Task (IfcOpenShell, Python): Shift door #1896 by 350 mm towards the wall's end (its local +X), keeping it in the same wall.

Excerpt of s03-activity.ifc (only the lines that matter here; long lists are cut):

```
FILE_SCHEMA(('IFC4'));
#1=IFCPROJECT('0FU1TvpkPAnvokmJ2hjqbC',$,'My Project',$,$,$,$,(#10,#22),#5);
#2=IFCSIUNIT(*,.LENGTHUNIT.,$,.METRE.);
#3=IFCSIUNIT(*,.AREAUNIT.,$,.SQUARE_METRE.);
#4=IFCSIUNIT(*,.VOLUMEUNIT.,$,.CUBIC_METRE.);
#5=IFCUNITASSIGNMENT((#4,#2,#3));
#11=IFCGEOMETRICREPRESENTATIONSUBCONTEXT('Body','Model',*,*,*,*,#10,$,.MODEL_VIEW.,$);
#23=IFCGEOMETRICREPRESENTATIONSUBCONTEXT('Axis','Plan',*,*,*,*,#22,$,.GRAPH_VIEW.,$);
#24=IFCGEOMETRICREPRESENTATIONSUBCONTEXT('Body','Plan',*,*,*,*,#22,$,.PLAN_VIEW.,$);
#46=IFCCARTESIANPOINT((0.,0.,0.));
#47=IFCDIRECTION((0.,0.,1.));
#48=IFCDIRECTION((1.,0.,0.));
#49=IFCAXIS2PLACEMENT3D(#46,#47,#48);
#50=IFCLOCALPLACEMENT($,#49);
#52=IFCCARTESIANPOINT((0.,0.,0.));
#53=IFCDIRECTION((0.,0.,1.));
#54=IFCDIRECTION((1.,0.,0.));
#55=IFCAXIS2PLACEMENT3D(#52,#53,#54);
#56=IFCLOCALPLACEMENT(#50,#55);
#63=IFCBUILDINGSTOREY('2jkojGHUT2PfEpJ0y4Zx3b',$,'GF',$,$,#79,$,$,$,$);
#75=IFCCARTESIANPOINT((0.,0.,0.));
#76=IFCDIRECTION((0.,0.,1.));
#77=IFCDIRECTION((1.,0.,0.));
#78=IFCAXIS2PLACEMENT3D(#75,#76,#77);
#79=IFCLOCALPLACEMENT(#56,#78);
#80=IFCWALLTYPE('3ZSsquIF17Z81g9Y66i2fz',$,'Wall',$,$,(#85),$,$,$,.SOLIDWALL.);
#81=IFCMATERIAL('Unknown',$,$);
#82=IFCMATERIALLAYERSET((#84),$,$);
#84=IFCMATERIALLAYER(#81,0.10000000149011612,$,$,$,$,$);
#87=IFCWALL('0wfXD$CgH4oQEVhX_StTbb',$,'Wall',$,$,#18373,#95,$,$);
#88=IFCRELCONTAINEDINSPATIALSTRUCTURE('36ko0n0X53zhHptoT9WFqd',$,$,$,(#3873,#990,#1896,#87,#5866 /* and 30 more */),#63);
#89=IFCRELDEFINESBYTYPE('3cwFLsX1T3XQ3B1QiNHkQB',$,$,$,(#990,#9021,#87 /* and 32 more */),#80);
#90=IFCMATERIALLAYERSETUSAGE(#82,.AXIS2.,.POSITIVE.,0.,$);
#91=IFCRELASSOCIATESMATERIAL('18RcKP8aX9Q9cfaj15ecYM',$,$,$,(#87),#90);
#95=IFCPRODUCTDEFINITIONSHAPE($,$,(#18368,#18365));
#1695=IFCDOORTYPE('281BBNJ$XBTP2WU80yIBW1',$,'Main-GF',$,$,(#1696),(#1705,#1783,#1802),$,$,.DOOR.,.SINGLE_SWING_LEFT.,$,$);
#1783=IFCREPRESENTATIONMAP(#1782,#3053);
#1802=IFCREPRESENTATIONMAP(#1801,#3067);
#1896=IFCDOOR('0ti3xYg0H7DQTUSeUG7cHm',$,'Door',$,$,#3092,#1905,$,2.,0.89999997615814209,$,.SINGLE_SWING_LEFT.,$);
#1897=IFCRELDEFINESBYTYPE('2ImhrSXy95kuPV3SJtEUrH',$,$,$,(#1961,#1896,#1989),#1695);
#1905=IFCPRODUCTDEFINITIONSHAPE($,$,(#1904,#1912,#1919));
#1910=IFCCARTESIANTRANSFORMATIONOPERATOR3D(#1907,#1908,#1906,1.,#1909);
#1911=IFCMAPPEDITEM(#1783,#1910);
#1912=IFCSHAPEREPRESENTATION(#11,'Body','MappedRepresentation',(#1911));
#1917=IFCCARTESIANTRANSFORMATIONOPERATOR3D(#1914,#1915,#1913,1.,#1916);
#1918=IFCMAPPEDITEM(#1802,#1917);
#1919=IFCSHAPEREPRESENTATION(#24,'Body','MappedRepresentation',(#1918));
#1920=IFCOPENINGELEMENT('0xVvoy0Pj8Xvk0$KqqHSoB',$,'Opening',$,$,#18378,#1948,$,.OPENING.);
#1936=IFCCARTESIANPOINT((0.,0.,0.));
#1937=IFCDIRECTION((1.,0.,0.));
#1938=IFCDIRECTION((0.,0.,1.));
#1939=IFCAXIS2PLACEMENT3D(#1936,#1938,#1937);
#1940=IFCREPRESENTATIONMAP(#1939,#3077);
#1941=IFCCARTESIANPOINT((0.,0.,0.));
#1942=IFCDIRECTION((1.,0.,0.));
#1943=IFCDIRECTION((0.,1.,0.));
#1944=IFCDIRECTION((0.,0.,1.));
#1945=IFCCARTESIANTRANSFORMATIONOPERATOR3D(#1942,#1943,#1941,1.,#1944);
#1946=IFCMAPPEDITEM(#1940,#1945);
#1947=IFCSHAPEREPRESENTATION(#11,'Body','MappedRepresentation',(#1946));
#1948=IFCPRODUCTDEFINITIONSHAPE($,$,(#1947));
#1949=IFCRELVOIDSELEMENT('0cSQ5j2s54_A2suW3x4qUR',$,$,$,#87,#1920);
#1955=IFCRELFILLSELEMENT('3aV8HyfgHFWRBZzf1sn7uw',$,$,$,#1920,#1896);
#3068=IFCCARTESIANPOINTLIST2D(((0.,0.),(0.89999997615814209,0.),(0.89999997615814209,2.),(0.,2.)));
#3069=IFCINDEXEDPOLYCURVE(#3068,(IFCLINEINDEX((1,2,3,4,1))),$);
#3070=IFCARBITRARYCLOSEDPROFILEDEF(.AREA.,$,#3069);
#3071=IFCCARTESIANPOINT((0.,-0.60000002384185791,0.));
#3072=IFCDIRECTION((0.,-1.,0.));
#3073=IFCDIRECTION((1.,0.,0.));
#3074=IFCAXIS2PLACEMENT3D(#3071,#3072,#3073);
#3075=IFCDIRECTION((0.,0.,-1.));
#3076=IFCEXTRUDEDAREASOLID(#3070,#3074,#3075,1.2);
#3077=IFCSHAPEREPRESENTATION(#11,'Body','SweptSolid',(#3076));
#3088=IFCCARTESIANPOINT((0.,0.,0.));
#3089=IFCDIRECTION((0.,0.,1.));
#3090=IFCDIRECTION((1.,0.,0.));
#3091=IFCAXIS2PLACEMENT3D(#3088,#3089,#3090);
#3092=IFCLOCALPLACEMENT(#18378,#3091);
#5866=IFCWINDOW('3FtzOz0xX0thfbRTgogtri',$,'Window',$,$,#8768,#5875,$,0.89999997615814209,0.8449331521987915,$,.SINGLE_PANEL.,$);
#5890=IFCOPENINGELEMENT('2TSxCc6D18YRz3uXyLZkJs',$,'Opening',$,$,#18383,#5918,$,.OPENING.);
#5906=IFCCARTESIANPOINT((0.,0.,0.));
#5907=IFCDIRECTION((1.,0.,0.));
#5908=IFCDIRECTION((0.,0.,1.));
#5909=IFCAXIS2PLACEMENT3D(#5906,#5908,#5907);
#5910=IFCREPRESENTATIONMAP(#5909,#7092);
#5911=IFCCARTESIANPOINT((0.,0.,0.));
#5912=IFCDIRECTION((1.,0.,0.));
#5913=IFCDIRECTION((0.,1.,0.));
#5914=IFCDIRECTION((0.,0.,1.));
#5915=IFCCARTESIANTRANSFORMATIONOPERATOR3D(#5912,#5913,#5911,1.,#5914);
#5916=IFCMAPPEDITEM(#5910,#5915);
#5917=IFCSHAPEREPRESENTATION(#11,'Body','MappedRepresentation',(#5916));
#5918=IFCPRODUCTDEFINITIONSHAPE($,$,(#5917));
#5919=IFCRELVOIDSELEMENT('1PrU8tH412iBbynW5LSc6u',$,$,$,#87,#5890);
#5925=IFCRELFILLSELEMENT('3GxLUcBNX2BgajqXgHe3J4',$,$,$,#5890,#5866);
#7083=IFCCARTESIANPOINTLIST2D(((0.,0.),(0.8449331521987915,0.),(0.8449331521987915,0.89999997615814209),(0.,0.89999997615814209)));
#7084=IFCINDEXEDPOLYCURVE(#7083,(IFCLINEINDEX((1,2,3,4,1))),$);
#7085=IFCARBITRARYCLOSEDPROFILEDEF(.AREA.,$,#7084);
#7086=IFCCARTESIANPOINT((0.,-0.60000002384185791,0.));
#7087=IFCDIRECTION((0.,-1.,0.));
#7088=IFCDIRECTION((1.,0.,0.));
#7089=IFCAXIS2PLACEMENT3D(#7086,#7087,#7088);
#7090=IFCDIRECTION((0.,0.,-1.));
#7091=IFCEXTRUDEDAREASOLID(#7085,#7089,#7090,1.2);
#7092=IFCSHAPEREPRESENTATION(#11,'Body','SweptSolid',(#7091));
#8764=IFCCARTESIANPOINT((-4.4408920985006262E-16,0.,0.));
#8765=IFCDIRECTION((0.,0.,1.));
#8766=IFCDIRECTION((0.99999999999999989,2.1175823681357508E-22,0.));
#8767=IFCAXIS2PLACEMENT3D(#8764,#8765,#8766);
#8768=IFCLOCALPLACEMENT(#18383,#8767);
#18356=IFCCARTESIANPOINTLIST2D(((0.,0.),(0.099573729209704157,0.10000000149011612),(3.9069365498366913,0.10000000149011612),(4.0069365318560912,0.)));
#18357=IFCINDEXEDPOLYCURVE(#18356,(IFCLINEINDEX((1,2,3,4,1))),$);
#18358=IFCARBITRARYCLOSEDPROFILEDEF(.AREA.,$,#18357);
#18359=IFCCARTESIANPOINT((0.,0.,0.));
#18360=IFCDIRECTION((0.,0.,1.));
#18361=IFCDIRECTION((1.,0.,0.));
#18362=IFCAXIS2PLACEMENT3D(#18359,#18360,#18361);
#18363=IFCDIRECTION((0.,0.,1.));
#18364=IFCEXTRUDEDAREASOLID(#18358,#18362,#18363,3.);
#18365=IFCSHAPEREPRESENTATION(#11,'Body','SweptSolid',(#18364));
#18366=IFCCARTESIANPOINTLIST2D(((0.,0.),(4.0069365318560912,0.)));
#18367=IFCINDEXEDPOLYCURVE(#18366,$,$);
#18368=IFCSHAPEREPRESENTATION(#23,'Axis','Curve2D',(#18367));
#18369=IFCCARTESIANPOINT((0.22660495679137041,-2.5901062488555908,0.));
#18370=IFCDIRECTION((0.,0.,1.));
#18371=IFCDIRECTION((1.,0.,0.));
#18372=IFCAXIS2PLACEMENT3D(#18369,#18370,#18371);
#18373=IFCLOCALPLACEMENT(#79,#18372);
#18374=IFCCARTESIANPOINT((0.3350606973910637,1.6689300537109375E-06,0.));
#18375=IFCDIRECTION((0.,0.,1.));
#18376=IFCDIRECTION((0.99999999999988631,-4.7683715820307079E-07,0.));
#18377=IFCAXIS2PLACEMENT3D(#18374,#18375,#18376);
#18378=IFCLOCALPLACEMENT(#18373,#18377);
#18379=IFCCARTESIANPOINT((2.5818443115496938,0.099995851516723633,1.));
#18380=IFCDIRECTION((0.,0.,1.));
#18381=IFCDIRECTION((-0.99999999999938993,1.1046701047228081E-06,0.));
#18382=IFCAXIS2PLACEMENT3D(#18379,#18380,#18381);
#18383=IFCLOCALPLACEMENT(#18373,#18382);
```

```python
import ifcopenshell
import ifcopenshell.api.geometry
import ifcopenshell.util.placement
import ifcopenshell.util.unit

model = ifcopenshell.open("s03-activity.ifc")
unit_scale = ifcopenshell.util.unit.calculate_unit_scale(model)

door = model.by_guid("0ti3xYg0H7DQTUSeUG7cHm")
opening = door.FillsVoids[0].RelatingOpeningElement
wall = opening.VoidsElements[0].RelatingBuildingElement

wall_matrix = ifcopenshell.util.placement.get_local_placement(wall.ObjectPlacement)
shift = wall_matrix[:3, 0] * 0.35 / unit_scale
before = ifcopenshell.util.placement.get_local_placement(door.ObjectPlacement)[:3, 3].copy()

# The door is placed relative to its opening, so it follows when the opening moves.
matrix = ifcopenshell.util.placement.get_local_placement(opening.ObjectPlacement)
matrix[:3, 3] += shift
ifcopenshell.api.geometry.edit_object_placement(
    model, product=opening, matrix=matrix, is_si=False, should_transform_children=True
)

after = ifcopenshell.util.placement.get_local_placement(door.ObjectPlacement)[:3, 3]
print("door moved by", (after - before).round(3) + 0.0)

model.write("s03-activity_updated.ifc")
```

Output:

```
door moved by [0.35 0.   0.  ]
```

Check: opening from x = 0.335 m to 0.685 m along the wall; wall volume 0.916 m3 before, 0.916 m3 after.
